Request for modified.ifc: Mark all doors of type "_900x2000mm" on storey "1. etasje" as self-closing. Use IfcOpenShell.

First a look at what the model holds.

```python
import ifcopenshell
import ifcopenshell.util.element

model = ifcopenshell.open("modified.ifc")
print(model.schema)
storey = next(s for s in model.by_type("IfcBuildingStorey") if s.Name == "1. etasje")
doors = [e for e in ifcopenshell.util.element.get_decomposition(storey) if e.is_a("IfcDoor")]
seen = {}
for e in doors:
    element_type = ifcopenshell.util.element.get_type(e)
    key = (element_type.Name if element_type != e and element_type else None, ifcopenshell.util.element.get_pset(e, "Pset_DoorCommon", "SelfClosing"))
    seen[key] = seen.get(key, 0) + 1
for (name, value), count in sorted(seen.items(), key=str):
    print(count, "x", name, "|", value)
```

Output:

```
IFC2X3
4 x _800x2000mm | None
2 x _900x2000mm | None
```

```python
import ifcopenshell
import ifcopenshell.api.pset
import ifcopenshell.util.element

model = ifcopenshell.open("modified.ifc")

storey = next(s for s in model.by_type("IfcBuildingStorey") if s.Name == "1. etasje")
doors = [e for e in ifcopenshell.util.element.get_decomposition(storey) if e.is_a("IfcDoor")]

count = 0
for e in doors:
    element_type = ifcopenshell.util.element.get_type(e)
    if element_type in (None, e) or element_type.Name != "_900x2000mm":
        continue
    # add_pset returns the element's existing set when there is one.
    pset = ifcopenshell.api.pset.add_pset(model, product=e, name="Pset_DoorCommon")
    ifcopenshell.api.pset.edit_pset(model, pset=pset, properties={"SelfClosing": True})
    count += 1

print(count, "doors updated")

model.write("modified-out.ifc")
```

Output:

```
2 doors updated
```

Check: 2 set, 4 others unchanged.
